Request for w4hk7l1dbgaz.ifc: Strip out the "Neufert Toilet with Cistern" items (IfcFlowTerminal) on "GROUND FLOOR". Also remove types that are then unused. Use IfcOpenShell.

First a look at what the model holds.

```python
import ifcopenshell
import ifcopenshell.util.element

model = ifcopenshell.open("w4hk7l1dbgaz.ifc")
print(model.schema)
storey = next(s for s in model.by_type("IfcBuildingStorey") if s.Name == "GROUND FLOOR")
terminals = [e for e in ifcopenshell.util.element.get_decomposition(storey) if e.is_a("IfcFlowTerminal")]
seen = {}
for e in terminals:
    element_type = ifcopenshell.util.element.get_type(e)
    name = element_type.Name if element_type not in (None, e) else None
    seen[name] = seen.get(name, 0) + 1
for name, count in sorted(seen.items(), key=str):
    print(count, "x", name)
```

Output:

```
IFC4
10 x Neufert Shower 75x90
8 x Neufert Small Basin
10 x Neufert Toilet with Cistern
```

```python
import ifcopenshell
import ifcopenshell.api.root
import ifcopenshell.util.element

model = ifcopenshell.open("w4hk7l1dbgaz.ifc")

storey = next(s for s in model.by_type("IfcBuildingStorey") if s.Name == "GROUND FLOOR")
terminals = [e for e in ifcopenshell.util.element.get_decomposition(storey) if e.is_a("IfcFlowTerminal")]
targets = [e for e in terminals if (t := ifcopenshell.util.element.get_type(e)) not in (None, e) and t.Name == "Neufert Toilet with Cistern"]
types = {ifcopenshell.util.element.get_type(e) for e in targets} - {None, *targets}

for e in targets:
    ifcopenshell.api.root.remove_product(model, product=e)
print(len(targets), "removed")

unused = [t for t in types if not ifcopenshell.util.element.get_types(t)]
for t in unused:
    ifcopenshell.api.root.remove_product(model, product=t)
print(len(unused), "unused types removed")

model.write("w4hk7l1dbgaz_v2.ifc")
```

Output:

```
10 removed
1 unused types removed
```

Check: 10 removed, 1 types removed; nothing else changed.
